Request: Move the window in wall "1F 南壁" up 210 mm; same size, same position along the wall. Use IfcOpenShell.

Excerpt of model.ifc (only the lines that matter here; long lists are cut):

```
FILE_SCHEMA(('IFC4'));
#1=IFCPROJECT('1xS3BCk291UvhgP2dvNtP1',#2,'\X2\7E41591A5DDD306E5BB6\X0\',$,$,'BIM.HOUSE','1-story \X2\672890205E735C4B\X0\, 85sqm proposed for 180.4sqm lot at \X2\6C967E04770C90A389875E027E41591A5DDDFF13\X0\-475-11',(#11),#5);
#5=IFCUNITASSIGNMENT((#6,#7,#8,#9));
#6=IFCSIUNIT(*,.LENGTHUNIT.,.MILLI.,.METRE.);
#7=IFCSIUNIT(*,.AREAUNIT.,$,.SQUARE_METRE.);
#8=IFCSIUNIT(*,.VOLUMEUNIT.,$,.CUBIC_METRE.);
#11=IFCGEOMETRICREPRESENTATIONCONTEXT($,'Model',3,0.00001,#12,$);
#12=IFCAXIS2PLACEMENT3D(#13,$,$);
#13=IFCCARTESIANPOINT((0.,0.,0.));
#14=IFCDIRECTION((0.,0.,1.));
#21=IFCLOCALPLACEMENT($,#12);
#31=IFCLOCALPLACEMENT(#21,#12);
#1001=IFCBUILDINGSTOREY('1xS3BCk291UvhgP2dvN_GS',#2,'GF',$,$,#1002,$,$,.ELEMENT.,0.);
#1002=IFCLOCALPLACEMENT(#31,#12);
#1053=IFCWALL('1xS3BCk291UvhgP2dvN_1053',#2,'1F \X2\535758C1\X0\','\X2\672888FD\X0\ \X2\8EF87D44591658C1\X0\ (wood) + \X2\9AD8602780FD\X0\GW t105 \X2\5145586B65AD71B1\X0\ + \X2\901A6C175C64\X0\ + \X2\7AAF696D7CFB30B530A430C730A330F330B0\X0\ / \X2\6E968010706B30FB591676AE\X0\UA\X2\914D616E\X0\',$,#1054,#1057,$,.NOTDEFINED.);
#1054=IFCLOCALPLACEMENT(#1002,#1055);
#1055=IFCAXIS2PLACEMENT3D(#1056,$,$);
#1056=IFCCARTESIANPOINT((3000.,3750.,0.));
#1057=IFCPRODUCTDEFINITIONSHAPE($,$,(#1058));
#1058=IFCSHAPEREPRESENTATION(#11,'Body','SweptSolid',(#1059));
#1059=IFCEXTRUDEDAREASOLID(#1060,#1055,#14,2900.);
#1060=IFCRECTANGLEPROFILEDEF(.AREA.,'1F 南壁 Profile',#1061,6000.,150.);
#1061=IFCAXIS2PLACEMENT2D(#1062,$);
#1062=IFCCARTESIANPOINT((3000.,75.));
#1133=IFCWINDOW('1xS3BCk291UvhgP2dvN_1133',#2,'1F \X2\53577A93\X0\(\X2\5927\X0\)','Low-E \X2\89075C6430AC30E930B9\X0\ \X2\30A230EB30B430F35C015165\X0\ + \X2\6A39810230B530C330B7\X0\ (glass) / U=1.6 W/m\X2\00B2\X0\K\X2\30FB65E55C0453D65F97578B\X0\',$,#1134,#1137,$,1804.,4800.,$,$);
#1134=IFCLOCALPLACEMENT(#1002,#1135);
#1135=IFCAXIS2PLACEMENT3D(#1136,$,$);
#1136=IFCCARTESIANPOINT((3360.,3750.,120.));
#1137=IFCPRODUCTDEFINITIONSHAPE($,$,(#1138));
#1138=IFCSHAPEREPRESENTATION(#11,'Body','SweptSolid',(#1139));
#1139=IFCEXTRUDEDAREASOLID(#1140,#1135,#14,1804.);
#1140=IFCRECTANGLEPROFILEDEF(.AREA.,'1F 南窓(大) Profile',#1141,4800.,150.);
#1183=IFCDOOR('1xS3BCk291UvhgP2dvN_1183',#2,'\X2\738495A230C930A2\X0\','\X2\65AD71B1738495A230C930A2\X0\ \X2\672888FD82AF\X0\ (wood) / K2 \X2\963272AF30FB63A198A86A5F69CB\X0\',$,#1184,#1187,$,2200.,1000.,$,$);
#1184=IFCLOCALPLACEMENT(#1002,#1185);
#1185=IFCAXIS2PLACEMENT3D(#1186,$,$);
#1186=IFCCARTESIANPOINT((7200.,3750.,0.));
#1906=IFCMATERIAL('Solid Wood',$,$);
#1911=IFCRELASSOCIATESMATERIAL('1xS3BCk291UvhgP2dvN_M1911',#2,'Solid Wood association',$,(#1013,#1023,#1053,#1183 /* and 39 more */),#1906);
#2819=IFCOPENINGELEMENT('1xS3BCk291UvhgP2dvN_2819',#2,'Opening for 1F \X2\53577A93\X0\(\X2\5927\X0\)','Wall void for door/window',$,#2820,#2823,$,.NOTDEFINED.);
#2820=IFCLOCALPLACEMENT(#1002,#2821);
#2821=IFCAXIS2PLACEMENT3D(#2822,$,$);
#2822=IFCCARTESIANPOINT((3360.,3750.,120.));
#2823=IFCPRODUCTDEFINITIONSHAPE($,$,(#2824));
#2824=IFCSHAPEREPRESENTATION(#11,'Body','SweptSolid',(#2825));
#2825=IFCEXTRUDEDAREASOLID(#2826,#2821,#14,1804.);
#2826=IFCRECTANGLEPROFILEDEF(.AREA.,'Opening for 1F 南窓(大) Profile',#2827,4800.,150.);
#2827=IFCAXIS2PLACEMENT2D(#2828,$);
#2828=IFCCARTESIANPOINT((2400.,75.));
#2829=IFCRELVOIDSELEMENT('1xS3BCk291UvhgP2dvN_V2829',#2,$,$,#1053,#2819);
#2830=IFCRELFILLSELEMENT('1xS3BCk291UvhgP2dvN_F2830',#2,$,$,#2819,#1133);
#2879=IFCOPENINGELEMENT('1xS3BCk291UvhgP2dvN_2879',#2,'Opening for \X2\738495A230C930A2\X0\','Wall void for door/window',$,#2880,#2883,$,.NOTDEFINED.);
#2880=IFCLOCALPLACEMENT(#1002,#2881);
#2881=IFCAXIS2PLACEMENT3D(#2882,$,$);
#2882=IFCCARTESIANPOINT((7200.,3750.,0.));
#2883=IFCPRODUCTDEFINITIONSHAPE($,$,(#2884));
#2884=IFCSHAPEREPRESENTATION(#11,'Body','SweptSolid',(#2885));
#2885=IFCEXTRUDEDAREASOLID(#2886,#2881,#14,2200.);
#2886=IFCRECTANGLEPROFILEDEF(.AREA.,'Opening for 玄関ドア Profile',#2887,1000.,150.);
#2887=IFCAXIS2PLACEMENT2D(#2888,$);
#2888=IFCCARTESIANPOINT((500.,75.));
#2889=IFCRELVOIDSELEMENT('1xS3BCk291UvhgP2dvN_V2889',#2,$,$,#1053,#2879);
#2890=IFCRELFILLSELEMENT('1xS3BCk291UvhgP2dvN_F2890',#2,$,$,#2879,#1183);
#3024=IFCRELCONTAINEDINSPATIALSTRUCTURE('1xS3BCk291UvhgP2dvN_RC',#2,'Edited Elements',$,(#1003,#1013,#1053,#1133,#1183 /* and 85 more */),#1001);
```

```python
import numpy as np
import ifcopenshell
import ifcopenshell.api.geometry
import ifcopenshell.util.placement
import ifcopenshell.util.unit

model = ifcopenshell.open("model.ifc")
unit_scale = ifcopenshell.util.unit.calculate_unit_scale(model)

window = model.by_guid("1xS3BCk291UvhgP2dvN_1133")
opening = window.FillsVoids[0].RelatingOpeningElement
dz = 210.0

shift = np.array([0.0, 0.0, dz])
# The window is not placed relative to its opening, so move both.
for product in (opening, window):
    matrix = ifcopenshell.util.placement.get_local_placement(product.ObjectPlacement)
    matrix[:3, 3] += shift
    ifcopenshell.api.geometry.edit_object_placement(model, product=product, matrix=matrix, is_si=False)

print(f"moved by {dz * unit_scale:+.3f} m")

model.write("model_rev.ifc")
```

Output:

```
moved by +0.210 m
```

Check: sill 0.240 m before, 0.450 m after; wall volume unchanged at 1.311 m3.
